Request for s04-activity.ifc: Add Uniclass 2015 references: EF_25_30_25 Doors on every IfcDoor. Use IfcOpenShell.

First a look at what the model holds.

```python
import ifcopenshell

model = ifcopenshell.open("s04-activity.ifc")
print(model.schema)
print("classifications:", [c.Name for c in model.by_type("IfcClassification")])
for ifc_class in ("IfcDoor", "IfcRoof", "IfcStair", "IfcWall", "IfcWindow"):
    print(ifc_class, len(model.by_type(ifc_class)))
```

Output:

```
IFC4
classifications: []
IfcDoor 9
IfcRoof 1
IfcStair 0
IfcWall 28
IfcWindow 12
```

```python
import ifcopenshell
import ifcopenshell.api.classification

model = ifcopenshell.open("s04-activity.ifc")

system = ifcopenshell.api.classification.add_classification(model, classification="Uniclass 2015")

codes = {
    "IfcDoor": ("EF_25_30_25", "Doors"),
}
for ifc_class, (code, name) in codes.items():
    products = model.by_type(ifc_class)
    ifcopenshell.api.classification.add_reference(
        model, products=products, classification=system, identification=code, name=name
    )
    print(code, len(products))

model.write("s04-activity_v2.ifc")
```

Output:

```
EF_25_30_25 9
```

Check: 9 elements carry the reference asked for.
